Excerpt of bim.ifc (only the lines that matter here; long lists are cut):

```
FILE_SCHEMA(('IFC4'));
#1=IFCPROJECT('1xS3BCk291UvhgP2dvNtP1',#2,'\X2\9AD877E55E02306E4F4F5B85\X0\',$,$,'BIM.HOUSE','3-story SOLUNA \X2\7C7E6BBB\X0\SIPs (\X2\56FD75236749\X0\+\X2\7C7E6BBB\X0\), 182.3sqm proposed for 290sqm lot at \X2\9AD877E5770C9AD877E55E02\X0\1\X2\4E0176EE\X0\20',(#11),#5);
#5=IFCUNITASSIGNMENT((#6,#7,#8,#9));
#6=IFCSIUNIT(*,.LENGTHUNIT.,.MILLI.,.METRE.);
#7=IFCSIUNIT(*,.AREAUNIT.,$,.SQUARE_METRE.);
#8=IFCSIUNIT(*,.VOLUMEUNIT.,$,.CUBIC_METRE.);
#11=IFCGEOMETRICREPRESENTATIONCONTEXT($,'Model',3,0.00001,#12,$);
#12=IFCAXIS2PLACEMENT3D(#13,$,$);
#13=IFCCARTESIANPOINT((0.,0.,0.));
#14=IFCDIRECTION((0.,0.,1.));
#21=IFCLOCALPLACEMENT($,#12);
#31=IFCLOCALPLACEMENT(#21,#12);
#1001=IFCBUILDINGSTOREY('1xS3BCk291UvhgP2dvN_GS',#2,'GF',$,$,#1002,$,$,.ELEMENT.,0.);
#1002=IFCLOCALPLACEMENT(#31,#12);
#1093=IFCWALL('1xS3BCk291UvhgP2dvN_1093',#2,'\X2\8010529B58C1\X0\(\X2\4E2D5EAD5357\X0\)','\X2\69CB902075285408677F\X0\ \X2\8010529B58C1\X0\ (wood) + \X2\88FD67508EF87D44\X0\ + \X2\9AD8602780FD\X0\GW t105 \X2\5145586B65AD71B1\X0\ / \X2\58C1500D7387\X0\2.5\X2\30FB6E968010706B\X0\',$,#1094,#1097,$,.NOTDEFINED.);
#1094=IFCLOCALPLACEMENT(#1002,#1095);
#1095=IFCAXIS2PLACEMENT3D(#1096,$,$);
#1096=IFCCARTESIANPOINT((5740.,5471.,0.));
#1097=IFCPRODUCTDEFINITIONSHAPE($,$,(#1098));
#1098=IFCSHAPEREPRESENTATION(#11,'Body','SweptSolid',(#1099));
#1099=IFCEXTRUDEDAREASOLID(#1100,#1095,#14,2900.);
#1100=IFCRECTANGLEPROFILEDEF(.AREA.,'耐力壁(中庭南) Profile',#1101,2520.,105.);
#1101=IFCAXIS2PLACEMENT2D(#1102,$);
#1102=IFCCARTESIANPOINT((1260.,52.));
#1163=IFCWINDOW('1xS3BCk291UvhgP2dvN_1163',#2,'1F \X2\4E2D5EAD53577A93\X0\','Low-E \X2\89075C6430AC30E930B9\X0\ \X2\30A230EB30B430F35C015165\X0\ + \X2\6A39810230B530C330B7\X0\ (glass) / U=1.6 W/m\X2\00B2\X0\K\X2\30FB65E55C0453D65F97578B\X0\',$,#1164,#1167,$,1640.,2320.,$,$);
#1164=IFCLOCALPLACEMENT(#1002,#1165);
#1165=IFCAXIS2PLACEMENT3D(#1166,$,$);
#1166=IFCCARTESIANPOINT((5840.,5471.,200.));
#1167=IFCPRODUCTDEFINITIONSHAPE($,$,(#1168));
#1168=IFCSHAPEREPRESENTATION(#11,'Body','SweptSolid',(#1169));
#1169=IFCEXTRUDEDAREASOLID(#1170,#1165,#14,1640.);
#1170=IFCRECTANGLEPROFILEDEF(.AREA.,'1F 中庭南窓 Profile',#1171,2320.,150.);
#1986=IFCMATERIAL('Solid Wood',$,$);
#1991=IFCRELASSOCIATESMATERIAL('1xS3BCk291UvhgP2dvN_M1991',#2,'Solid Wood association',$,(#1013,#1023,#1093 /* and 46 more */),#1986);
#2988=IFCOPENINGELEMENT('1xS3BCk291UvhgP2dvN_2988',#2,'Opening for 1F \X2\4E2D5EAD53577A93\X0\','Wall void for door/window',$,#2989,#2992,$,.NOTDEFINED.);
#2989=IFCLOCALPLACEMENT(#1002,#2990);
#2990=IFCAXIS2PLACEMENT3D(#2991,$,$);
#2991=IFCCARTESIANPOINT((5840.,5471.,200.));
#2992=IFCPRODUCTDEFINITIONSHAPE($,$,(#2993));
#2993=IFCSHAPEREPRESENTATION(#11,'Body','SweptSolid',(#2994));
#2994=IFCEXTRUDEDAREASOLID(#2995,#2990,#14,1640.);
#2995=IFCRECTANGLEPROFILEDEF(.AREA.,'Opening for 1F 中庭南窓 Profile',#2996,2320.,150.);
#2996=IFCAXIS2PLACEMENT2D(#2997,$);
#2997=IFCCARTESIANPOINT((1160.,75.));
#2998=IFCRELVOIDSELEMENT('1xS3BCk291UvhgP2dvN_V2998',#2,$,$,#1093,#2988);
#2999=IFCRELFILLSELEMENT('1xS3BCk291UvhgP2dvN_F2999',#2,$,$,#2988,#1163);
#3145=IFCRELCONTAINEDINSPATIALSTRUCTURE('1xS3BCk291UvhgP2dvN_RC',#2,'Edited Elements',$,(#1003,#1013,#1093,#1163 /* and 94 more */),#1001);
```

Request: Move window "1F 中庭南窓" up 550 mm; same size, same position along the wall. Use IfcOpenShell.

```python
import numpy as np
import ifcopenshell
import ifcopenshell.api.geometry
import ifcopenshell.util.placement
import ifcopenshell.util.unit

model = ifcopenshell.open("bim.ifc")
unit_scale = ifcopenshell.util.unit.calculate_unit_scale(model)

window = model.by_guid("1xS3BCk291UvhgP2dvN_1163")
opening = window.FillsVoids[0].RelatingOpeningElement
dz = 550.0

shift = np.array([0.0, 0.0, dz])
# The window is not placed relative to its opening, so move both.
for product in (opening, window):
    matrix = ifcopenshell.util.placement.get_local_placement(product.ObjectPlacement)
    matrix[:3, 3] += shift
    ifcopenshell.api.geometry.edit_object_placement(model, product=product, matrix=matrix, is_si=False)

print(f"moved by {dz * unit_scale:+.3f} m")

model.write("bim_rev.ifc")
```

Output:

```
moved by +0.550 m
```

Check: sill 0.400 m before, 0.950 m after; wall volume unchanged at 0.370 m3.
